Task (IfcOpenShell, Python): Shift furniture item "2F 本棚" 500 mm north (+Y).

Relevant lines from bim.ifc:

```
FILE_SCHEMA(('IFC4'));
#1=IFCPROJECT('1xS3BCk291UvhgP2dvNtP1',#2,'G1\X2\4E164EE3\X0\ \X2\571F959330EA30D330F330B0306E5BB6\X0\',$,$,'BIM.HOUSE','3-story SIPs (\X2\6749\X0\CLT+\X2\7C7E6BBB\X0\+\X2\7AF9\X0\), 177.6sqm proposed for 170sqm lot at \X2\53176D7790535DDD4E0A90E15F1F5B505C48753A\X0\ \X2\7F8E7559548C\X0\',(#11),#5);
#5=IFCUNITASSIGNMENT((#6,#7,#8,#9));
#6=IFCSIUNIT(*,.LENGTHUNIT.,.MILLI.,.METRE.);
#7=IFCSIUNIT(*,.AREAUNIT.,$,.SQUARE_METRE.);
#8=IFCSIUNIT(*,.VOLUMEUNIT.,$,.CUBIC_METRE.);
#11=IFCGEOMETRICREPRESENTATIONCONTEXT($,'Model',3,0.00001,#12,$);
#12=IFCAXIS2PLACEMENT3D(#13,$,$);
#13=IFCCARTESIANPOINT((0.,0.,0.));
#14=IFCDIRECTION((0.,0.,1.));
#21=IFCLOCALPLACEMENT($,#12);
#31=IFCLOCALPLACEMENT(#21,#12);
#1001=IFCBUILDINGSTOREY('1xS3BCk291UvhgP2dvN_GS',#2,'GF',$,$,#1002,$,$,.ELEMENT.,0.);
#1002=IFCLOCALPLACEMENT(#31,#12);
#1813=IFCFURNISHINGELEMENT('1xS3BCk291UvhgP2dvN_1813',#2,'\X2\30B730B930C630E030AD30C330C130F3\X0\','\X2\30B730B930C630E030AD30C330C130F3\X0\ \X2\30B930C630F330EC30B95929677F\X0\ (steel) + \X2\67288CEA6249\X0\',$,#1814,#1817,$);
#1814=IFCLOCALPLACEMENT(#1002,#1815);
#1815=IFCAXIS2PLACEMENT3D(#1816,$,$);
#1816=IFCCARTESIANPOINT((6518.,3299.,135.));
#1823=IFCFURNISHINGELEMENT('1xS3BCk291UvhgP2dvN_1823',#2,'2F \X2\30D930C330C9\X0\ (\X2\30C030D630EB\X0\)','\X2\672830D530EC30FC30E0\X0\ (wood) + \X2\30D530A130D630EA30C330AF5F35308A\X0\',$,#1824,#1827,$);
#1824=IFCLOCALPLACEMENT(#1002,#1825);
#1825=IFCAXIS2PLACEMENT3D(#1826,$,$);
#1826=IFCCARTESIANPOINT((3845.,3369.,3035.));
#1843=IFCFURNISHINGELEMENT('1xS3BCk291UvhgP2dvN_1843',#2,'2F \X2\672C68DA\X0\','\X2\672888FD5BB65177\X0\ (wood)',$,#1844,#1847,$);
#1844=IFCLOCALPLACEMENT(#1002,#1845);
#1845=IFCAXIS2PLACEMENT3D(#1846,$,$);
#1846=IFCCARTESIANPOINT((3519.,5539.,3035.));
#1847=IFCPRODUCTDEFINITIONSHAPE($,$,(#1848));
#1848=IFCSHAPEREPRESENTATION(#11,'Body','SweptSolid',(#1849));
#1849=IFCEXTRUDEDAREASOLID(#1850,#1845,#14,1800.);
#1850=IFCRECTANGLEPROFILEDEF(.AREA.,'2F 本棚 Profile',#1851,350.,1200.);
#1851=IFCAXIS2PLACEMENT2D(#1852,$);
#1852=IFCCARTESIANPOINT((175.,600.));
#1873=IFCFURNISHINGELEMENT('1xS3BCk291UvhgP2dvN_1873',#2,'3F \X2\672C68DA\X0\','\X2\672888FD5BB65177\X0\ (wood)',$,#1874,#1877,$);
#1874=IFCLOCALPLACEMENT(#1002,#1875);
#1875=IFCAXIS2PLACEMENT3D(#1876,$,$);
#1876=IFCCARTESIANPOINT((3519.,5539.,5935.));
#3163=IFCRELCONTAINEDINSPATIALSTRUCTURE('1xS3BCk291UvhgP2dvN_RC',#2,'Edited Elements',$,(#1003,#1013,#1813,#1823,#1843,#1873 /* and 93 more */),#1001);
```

```python
import ifcopenshell
import ifcopenshell.api.geometry
import ifcopenshell.util.placement
import ifcopenshell.util.unit

model = ifcopenshell.open("bim.ifc")
unit_scale = ifcopenshell.util.unit.calculate_unit_scale(model)

item = model.by_guid("1xS3BCk291UvhgP2dvN_1843")
matrix = ifcopenshell.util.placement.get_local_placement(item.ObjectPlacement)
matrix[1, 3] += 0.5 / unit_scale
ifcopenshell.api.geometry.edit_object_placement(model, product=item, matrix=matrix, is_si=False)

print(ifcopenshell.util.placement.get_local_placement(item.ObjectPlacement).round(3) + 0.0)

model.write("bim_updated.ifc")
```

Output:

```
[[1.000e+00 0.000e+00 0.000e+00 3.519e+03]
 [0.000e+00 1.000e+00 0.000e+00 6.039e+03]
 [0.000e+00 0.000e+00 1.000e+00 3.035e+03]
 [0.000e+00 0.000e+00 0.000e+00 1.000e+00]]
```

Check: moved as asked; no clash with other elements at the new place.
